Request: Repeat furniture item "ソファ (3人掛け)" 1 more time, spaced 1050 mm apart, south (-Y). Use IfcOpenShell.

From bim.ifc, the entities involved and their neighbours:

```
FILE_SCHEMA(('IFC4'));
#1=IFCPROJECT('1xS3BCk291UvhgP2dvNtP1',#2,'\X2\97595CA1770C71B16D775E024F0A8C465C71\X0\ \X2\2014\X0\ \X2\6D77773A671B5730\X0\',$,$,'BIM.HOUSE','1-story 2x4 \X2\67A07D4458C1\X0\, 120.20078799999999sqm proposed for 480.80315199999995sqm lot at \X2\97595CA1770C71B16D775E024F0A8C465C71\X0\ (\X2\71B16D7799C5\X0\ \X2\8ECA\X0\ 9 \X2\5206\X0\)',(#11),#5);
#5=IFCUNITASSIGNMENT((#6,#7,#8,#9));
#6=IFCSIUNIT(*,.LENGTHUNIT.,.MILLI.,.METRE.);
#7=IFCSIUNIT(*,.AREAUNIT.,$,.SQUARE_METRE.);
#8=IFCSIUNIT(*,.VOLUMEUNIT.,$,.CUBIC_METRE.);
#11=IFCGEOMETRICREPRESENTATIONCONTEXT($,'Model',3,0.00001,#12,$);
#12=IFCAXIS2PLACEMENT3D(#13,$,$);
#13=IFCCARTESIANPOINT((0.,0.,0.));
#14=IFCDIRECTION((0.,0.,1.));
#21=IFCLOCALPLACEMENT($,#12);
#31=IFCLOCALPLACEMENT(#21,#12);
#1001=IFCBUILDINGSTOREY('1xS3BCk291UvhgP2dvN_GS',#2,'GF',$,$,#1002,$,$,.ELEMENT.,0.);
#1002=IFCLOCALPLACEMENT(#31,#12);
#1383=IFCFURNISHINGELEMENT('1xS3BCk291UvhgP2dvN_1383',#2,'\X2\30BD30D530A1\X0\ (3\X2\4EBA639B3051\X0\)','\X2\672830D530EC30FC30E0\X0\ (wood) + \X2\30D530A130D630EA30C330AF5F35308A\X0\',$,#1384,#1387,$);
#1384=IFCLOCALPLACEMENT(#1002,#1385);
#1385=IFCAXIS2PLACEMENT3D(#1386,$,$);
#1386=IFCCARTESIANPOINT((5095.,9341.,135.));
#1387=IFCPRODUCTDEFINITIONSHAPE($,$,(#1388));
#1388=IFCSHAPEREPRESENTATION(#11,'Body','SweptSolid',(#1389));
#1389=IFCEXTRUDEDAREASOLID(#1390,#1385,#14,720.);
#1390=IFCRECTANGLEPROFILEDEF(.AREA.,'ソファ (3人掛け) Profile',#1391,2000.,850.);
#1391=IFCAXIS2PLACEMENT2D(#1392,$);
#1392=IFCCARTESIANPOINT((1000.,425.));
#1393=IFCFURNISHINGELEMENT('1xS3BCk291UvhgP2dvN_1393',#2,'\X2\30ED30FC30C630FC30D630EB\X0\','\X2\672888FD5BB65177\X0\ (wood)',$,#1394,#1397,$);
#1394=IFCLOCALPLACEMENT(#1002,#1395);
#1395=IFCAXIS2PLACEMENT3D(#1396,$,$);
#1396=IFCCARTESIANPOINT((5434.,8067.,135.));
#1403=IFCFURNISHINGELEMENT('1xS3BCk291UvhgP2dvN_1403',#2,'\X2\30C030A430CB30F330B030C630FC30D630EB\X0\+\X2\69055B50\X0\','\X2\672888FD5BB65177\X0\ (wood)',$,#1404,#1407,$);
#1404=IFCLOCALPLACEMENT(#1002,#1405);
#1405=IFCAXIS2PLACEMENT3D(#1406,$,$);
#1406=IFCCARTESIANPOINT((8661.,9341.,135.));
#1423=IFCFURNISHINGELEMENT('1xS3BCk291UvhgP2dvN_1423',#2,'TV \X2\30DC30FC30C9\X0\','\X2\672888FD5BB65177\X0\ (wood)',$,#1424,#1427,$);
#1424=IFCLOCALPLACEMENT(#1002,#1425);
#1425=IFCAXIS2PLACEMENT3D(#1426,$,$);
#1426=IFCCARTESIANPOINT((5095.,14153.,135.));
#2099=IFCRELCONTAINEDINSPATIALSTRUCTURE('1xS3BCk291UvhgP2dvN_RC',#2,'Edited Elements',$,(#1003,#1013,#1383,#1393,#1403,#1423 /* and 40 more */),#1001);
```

```python
import numpy as np
import ifcopenshell
import ifcopenshell.api.geometry
import ifcopenshell.api.root
import ifcopenshell.util.element
import ifcopenshell.util.placement
import ifcopenshell.util.unit

model = ifcopenshell.open("bim.ifc")
unit_scale = ifcopenshell.util.unit.calculate_unit_scale(model)


def reuse_history(source, copy):
    """copy_class also copies each property set's owner history, people and application; keep the originals."""
    for rel in copy.IsDefinedBy:
        if rel.is_a("IfcRelDefinesByProperties") and (history := rel.RelatingPropertyDefinition.OwnerHistory):
            rel.RelatingPropertyDefinition.OwnerHistory = source.OwnerHistory
            ifcopenshell.util.element.remove_deep2(model, history)


source = model.by_guid("1xS3BCk291UvhgP2dvN_1383")
base = ifcopenshell.util.placement.get_local_placement(source.ObjectPlacement)
step = np.array([0.0, -1.0, 0.0]) * 1.05 / unit_scale

for i in range(1, 2):
    copy = ifcopenshell.api.root.copy_class(model, product=source)
    copy.Representation = ifcopenshell.util.element.copy_deep(
        model, source.Representation, exclude=["IfcGeometricRepresentationContext", "IfcRepresentationMap"]
    )
    reuse_history(source, copy)
    matrix = base.copy()
    matrix[:3, 3] += i * step
    print("added at", matrix[:3, 3].round(3) + 0.0)
    ifcopenshell.api.geometry.edit_object_placement(model, product=copy, matrix=matrix, is_si=False)

model.write("bim_edited.ifc")
```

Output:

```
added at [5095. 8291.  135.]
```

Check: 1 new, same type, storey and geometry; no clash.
